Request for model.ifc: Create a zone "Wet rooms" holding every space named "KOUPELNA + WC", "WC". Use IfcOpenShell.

First a look at what the model holds.

```python
import ifcopenshell

model = ifcopenshell.open("model.ifc")
print(model.schema)
seen = {}
for space in model.by_type("IfcSpace"):
    seen[space.LongName] = seen.get(space.LongName, 0) + 1
for name, count in sorted(seen.items(), key=str):
    print(count, "x", name)
print("zones:", [z.Name for z in model.by_type("IfcZone")][:20])
```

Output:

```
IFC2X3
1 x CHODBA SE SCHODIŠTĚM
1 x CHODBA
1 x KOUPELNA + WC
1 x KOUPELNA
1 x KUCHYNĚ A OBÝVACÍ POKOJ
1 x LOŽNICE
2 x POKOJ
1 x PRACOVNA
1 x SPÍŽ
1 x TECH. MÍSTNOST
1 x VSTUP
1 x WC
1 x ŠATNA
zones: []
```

```python
import ifcopenshell
import ifcopenshell.api.group
import ifcopenshell.api.root

model = ifcopenshell.open("model.ifc")

names = {"KOUPELNA + WC", "WC"}
spaces = [s for s in model.by_type("IfcSpace") if s.LongName in names]

zone = ifcopenshell.api.root.create_entity(model, ifc_class="IfcZone", name="Wet rooms")
ifcopenshell.api.group.assign_group(model, products=spaces, group=zone)
print(len(spaces), "spaces in", zone.Name)

model.write("model_updated.ifc")
```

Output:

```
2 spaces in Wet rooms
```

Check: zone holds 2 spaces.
